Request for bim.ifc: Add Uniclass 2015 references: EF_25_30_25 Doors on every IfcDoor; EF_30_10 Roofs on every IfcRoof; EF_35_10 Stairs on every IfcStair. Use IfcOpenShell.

First a look at what the model holds.

```python
import ifcopenshell

model = ifcopenshell.open("bim.ifc")
print(model.schema)
print("classifications:", [c.Name for c in model.by_type("IfcClassification")])
for ifc_class in ("IfcDoor", "IfcRoof", "IfcStair", "IfcWall", "IfcWindow"):
    print(ifc_class, len(model.by_type(ifc_class)))
```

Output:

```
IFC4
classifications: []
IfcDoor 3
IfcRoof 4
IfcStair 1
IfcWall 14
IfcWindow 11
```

```python
import ifcopenshell
import ifcopenshell.api.classification

model = ifcopenshell.open("bim.ifc")

system = ifcopenshell.api.classification.add_classification(model, classification="Uniclass 2015")

codes = {
    "IfcDoor": ("EF_25_30_25", "Doors"),
    "IfcRoof": ("EF_30_10", "Roofs"),
    "IfcStair": ("EF_35_10", "Stairs"),
}
for ifc_class, (code, name) in codes.items():
    products = model.by_type(ifc_class)
    ifcopenshell.api.classification.add_reference(
        model, products=products, classification=system, identification=code, name=name
    )
    print(code, len(products))

model.write("bim-out.ifc")
```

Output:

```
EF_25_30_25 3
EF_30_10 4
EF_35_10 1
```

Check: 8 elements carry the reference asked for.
